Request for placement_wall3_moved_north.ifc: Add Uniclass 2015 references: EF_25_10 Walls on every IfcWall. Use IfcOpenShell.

First a look at what the model holds.

```python
import ifcopenshell

model = ifcopenshell.open("placement_wall3_moved_north.ifc")
print(model.schema)
print("classifications:", [c.Name for c in model.by_type("IfcClassification")])
for ifc_class in ("IfcDoor", "IfcRoof", "IfcStair", "IfcWall", "IfcWindow"):
    print(ifc_class, len(model.by_type(ifc_class)))
```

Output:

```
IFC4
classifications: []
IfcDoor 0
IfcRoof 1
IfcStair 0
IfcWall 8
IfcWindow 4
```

```python
import ifcopenshell
import ifcopenshell.api.classification

model = ifcopenshell.open("placement_wall3_moved_north.ifc")

system = ifcopenshell.api.classification.add_classification(model, classification="Uniclass 2015")

codes = {
    "IfcWall": ("EF_25_10", "Walls"),
}
for ifc_class, (code, name) in codes.items():
    products = model.by_type(ifc_class)
    ifcopenshell.api.classification.add_reference(
        model, products=products, classification=system, identification=code, name=name
    )
    print(code, len(products))

model.write("placement_wall3_moved_north_v2.ifc")
```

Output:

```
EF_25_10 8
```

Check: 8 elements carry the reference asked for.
